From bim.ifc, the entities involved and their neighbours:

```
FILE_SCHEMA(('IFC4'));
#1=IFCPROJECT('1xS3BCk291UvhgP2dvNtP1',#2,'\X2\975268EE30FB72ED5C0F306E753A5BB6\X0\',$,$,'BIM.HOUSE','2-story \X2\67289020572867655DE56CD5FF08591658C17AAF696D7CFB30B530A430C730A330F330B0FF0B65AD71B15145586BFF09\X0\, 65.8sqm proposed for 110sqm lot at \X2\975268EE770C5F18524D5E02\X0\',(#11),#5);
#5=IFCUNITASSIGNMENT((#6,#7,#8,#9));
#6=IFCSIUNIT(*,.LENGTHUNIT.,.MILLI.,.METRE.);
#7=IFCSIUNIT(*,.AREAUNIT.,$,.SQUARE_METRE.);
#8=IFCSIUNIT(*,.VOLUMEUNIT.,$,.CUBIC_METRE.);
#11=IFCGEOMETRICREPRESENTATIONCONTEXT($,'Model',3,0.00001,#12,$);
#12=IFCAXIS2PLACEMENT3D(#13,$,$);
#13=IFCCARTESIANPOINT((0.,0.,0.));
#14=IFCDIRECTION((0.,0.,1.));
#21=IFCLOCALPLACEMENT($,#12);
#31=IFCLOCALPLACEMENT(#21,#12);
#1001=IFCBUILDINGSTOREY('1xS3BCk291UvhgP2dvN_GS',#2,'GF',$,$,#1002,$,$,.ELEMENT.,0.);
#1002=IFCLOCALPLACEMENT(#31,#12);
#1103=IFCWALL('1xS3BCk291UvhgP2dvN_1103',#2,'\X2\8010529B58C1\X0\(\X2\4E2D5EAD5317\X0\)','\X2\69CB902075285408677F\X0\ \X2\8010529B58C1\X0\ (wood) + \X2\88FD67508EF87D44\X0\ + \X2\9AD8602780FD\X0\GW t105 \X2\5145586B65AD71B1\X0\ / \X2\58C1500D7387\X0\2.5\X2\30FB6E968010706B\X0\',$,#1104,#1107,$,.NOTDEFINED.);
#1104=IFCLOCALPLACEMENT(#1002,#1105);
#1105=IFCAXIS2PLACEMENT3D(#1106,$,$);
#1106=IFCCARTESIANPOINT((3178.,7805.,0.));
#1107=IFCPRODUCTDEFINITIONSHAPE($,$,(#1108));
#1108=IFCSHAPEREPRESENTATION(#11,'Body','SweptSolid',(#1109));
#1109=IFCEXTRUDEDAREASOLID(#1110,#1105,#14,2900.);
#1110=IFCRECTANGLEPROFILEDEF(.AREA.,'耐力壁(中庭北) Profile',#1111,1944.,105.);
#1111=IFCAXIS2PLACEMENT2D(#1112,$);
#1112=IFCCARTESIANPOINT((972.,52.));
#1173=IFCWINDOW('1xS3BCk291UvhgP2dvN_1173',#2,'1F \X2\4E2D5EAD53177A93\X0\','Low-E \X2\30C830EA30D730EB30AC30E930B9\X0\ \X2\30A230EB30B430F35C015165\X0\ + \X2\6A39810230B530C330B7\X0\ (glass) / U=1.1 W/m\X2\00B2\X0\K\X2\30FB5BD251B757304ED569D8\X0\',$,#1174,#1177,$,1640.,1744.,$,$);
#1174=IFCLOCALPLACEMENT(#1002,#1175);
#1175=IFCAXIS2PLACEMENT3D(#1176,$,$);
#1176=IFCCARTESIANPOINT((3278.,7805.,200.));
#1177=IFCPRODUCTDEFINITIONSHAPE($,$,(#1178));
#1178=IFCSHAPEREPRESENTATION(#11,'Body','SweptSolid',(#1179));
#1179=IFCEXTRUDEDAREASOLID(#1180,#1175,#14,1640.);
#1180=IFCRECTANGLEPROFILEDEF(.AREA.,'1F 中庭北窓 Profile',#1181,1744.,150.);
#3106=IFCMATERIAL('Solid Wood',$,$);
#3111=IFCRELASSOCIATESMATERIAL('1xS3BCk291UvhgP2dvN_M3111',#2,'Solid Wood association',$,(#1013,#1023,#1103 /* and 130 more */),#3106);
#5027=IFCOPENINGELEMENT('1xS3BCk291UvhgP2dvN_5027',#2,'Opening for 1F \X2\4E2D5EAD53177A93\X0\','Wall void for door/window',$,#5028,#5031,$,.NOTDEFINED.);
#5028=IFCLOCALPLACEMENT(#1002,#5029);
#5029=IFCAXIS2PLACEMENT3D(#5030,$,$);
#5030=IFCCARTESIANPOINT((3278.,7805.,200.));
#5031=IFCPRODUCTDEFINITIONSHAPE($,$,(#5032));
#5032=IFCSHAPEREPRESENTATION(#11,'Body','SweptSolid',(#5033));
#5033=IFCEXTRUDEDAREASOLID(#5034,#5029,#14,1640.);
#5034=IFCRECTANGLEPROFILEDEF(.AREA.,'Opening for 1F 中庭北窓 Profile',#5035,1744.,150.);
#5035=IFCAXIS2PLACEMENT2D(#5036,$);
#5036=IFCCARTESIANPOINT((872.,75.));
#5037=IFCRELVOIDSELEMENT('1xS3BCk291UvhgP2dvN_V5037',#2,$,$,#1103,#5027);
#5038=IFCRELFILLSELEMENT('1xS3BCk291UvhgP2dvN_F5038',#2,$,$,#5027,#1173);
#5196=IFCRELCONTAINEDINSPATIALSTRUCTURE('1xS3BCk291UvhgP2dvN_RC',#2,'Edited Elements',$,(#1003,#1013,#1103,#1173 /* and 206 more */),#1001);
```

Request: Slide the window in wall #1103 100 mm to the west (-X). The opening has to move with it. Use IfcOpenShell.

```python
import ifcopenshell
import ifcopenshell.api.geometry
import ifcopenshell.util.placement
import ifcopenshell.util.unit

model = ifcopenshell.open("bim.ifc")
unit_scale = ifcopenshell.util.unit.calculate_unit_scale(model)

window = model.by_guid("1xS3BCk291UvhgP2dvN_1173")
opening = window.FillsVoids[0].RelatingOpeningElement
wall = opening.VoidsElements[0].RelatingBuildingElement

wall_matrix = ifcopenshell.util.placement.get_local_placement(wall.ObjectPlacement)
shift = wall_matrix[:3, 0] * -0.1 / unit_scale
before = ifcopenshell.util.placement.get_local_placement(window.ObjectPlacement)[:3, 3].copy()

# The window is not placed relative to its opening, so move both.
for product in (opening, window):
    matrix = ifcopenshell.util.placement.get_local_placement(product.ObjectPlacement)
    matrix[:3, 3] += shift
    ifcopenshell.api.geometry.edit_object_placement(model, product=product, matrix=matrix, is_si=False)

after = ifcopenshell.util.placement.get_local_placement(window.ObjectPlacement)[:3, 3]
print("window moved by", (after - before).round(3) + 0.0)

model.write("bim_updated.ifc")
```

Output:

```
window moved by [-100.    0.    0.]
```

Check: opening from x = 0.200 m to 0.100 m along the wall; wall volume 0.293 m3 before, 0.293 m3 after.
